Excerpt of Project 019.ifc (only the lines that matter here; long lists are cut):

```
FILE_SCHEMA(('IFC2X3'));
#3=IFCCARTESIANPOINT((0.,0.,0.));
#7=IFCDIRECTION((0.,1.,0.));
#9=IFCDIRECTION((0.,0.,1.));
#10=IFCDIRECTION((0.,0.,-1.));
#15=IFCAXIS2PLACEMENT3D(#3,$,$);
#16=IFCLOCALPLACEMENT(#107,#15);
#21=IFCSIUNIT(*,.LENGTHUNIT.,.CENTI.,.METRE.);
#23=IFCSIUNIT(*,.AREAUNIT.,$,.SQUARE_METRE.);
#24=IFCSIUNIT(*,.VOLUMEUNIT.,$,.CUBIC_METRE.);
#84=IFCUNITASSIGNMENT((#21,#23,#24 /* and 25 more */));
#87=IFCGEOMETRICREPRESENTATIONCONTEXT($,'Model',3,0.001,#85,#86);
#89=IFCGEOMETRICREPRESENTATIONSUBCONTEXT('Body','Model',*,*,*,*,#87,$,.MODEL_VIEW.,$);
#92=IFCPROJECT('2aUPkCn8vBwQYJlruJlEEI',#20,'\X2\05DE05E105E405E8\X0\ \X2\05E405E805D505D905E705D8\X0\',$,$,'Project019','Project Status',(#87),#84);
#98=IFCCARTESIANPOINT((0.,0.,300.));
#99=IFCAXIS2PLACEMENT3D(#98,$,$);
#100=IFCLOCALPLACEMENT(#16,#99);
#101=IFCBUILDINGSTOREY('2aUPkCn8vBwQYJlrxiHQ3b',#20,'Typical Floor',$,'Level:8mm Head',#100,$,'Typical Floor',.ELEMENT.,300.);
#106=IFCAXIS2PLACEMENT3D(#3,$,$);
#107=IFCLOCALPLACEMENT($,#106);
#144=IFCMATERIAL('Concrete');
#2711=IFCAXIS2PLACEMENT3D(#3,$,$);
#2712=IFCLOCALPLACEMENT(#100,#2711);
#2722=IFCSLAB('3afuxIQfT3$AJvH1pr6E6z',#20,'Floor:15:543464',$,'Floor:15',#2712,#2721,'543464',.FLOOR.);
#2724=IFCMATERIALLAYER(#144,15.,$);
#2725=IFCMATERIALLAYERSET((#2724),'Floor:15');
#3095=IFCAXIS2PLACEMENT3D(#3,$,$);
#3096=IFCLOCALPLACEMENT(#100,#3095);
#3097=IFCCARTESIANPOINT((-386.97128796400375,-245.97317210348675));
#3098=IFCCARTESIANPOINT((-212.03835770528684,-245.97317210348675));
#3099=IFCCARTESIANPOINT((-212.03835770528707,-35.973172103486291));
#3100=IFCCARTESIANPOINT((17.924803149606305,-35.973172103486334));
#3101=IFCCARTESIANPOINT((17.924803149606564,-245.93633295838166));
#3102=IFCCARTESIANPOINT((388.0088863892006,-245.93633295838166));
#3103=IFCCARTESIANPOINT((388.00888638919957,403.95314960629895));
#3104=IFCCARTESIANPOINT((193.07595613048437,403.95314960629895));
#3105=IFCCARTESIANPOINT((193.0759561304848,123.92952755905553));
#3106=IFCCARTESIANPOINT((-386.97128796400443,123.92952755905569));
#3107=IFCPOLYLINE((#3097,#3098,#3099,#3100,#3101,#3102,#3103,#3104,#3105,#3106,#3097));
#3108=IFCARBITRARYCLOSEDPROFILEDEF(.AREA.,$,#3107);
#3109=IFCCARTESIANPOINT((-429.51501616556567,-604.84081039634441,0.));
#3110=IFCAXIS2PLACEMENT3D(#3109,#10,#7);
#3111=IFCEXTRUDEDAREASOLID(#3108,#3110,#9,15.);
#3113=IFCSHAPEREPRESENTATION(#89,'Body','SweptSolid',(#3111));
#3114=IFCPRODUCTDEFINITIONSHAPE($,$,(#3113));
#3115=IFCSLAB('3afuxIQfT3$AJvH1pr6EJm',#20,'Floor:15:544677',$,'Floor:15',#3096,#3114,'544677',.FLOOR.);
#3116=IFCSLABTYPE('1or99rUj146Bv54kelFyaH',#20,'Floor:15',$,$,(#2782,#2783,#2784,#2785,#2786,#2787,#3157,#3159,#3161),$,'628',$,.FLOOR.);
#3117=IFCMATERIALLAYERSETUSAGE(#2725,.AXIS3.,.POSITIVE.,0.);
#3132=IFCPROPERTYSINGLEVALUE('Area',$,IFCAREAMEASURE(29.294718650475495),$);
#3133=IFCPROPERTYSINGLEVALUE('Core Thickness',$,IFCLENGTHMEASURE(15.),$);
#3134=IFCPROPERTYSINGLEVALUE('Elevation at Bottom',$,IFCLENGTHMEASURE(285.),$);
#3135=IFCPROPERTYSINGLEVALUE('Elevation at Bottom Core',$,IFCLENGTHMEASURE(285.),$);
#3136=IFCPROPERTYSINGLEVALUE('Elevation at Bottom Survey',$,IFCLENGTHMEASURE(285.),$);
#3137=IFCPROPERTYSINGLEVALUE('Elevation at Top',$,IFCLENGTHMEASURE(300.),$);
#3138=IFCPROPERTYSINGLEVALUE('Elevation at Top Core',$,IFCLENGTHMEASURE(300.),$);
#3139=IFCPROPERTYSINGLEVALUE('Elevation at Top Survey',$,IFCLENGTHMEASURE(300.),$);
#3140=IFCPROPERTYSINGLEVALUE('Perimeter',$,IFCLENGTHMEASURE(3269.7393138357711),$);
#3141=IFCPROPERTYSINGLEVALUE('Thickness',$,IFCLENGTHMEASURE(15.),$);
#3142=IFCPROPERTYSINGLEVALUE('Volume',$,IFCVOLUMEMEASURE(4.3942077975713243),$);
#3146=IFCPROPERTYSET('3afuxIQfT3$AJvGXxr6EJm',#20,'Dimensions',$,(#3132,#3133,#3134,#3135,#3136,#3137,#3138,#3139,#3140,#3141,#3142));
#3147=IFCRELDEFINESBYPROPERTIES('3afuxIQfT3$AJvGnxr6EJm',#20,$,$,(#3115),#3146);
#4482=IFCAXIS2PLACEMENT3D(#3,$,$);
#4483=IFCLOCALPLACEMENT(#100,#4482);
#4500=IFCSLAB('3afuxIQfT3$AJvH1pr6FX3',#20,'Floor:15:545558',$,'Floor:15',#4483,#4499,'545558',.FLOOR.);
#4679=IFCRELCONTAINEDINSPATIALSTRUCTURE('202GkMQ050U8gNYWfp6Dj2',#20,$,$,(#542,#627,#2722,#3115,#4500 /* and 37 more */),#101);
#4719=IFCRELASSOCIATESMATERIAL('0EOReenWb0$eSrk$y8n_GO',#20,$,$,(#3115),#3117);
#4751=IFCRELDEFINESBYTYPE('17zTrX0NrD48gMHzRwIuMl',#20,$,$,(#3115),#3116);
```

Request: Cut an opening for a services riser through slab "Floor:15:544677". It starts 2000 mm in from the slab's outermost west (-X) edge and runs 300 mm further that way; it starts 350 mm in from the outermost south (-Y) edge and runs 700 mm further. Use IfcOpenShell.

```python
import numpy as np
import ifcopenshell
import ifcopenshell.api.feature
import ifcopenshell.api.geometry
import ifcopenshell.api.pset
import ifcopenshell.api.root
import ifcopenshell.geom
import ifcopenshell.util.element
import ifcopenshell.util.placement
import ifcopenshell.util.representation
import ifcopenshell.util.shape
import ifcopenshell.util.unit

model = ifcopenshell.open("Project 019.ifc")
unit_scale = ifcopenshell.util.unit.calculate_unit_scale(model)
area_scale = ifcopenshell.util.unit.calculate_unit_scale(model, "AREAUNIT")
volume_scale = ifcopenshell.util.unit.calculate_unit_scale(model, "VOLUMEUNIT")
settings = ifcopenshell.geom.settings()


def volume(element):
    """Net volume in cubic metres, openings subtracted."""
    shape = ifcopenshell.geom.create_shape(settings, element)
    return ifcopenshell.util.shape.get_volume(shape.geometry)


slab = model.by_id(3115)
before = volume(slab)

# Extent in the slab's own axes, in metres. The edges named are its -X and -Y sides.
slab_shape = ifcopenshell.geom.create_shape(settings, slab)
vertices = ifcopenshell.util.shape.get_vertices(slab_shape.geometry)
x_min, y_min, bottom = vertices.min(axis=0)
top = vertices[:, 2].max()

opening = ifcopenshell.api.root.create_entity(model, ifc_class="IfcOpeningElement", name="Services riser opening")
context = ifcopenshell.util.representation.get_context(model, "Model", "Body", "MODEL_VIEW")
width, depth = 0.3, 0.7
outline = [(0.0, 0.0), (width, 0.0), (width, depth), (0.0, depth), (0.0, 0.0)]
# Overshoot both faces by 50 mm so the cut is clean.
shape = ifcopenshell.api.geometry.add_slab_representation(
    model, context=context, depth=top - bottom + 0.1, polyline=outline
)
ifcopenshell.api.geometry.assign_representation(model, product=opening, representation=shape)

matrix = ifcopenshell.util.placement.get_local_placement(slab.ObjectPlacement)
matrix[:, 3] = matrix @ np.append(np.array([x_min + 2, y_min + 0.35, bottom - 0.05]) / unit_scale, 1.0)
ifcopenshell.api.geometry.edit_object_placement(model, product=opening, matrix=matrix, is_si=False)
ifcopenshell.api.feature.add_feature(model, feature=opening, element=slab)

after = volume(slab)

# Update the slab's stored quantities.
pset = model.by_id(ifcopenshell.util.element.get_pset(slab, "Dimensions", should_inherit=False)["id"])
ifcopenshell.api.pset.edit_pset(model, pset=pset, properties={
    "Area": model.create_entity("IfcAreaMeasure", after / (top - bottom) / area_scale),
    "Volume": model.create_entity("IfcVolumeMeasure", after / volume_scale),
})

print(f"slab volume {before:.3f} -> {after:.3f} m3")

model.write("Project 019_updated.ifc")
```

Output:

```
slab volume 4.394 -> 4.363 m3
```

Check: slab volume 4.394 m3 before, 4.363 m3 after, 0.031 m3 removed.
